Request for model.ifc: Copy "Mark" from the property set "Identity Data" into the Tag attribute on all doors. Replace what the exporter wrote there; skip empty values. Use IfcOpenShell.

First a look at what the model holds.

```python
import ifcopenshell
import ifcopenshell.util.element

model = ifcopenshell.open("model.ifc")
print(model.schema)
doors = model.by_type("IfcDoor")
print(len(doors), "doors")
for e in doors[:8]:
    source = ifcopenshell.util.element.get_pset(e, "Identity Data", "Mark")
    target = e.Tag
    print(e.id(), repr(source), repr(target), sep=" | ")
```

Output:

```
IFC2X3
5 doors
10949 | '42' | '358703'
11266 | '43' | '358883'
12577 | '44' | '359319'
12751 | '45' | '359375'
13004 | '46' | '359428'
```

```python
import ifcopenshell
import ifcopenshell.util.element

model = ifcopenshell.open("model.ifc")

count = 0
for e in model.by_type("IfcDoor"):
    value = ifcopenshell.util.element.get_pset(e, "Identity Data", "Mark")
    current = e.Tag
    if not value or not value.strip() or current == value:
        continue
    e.Tag = value
    count += 1

print(count, "doors updated")

model.write("model_edited.ifc")
```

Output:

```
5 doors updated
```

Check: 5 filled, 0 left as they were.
